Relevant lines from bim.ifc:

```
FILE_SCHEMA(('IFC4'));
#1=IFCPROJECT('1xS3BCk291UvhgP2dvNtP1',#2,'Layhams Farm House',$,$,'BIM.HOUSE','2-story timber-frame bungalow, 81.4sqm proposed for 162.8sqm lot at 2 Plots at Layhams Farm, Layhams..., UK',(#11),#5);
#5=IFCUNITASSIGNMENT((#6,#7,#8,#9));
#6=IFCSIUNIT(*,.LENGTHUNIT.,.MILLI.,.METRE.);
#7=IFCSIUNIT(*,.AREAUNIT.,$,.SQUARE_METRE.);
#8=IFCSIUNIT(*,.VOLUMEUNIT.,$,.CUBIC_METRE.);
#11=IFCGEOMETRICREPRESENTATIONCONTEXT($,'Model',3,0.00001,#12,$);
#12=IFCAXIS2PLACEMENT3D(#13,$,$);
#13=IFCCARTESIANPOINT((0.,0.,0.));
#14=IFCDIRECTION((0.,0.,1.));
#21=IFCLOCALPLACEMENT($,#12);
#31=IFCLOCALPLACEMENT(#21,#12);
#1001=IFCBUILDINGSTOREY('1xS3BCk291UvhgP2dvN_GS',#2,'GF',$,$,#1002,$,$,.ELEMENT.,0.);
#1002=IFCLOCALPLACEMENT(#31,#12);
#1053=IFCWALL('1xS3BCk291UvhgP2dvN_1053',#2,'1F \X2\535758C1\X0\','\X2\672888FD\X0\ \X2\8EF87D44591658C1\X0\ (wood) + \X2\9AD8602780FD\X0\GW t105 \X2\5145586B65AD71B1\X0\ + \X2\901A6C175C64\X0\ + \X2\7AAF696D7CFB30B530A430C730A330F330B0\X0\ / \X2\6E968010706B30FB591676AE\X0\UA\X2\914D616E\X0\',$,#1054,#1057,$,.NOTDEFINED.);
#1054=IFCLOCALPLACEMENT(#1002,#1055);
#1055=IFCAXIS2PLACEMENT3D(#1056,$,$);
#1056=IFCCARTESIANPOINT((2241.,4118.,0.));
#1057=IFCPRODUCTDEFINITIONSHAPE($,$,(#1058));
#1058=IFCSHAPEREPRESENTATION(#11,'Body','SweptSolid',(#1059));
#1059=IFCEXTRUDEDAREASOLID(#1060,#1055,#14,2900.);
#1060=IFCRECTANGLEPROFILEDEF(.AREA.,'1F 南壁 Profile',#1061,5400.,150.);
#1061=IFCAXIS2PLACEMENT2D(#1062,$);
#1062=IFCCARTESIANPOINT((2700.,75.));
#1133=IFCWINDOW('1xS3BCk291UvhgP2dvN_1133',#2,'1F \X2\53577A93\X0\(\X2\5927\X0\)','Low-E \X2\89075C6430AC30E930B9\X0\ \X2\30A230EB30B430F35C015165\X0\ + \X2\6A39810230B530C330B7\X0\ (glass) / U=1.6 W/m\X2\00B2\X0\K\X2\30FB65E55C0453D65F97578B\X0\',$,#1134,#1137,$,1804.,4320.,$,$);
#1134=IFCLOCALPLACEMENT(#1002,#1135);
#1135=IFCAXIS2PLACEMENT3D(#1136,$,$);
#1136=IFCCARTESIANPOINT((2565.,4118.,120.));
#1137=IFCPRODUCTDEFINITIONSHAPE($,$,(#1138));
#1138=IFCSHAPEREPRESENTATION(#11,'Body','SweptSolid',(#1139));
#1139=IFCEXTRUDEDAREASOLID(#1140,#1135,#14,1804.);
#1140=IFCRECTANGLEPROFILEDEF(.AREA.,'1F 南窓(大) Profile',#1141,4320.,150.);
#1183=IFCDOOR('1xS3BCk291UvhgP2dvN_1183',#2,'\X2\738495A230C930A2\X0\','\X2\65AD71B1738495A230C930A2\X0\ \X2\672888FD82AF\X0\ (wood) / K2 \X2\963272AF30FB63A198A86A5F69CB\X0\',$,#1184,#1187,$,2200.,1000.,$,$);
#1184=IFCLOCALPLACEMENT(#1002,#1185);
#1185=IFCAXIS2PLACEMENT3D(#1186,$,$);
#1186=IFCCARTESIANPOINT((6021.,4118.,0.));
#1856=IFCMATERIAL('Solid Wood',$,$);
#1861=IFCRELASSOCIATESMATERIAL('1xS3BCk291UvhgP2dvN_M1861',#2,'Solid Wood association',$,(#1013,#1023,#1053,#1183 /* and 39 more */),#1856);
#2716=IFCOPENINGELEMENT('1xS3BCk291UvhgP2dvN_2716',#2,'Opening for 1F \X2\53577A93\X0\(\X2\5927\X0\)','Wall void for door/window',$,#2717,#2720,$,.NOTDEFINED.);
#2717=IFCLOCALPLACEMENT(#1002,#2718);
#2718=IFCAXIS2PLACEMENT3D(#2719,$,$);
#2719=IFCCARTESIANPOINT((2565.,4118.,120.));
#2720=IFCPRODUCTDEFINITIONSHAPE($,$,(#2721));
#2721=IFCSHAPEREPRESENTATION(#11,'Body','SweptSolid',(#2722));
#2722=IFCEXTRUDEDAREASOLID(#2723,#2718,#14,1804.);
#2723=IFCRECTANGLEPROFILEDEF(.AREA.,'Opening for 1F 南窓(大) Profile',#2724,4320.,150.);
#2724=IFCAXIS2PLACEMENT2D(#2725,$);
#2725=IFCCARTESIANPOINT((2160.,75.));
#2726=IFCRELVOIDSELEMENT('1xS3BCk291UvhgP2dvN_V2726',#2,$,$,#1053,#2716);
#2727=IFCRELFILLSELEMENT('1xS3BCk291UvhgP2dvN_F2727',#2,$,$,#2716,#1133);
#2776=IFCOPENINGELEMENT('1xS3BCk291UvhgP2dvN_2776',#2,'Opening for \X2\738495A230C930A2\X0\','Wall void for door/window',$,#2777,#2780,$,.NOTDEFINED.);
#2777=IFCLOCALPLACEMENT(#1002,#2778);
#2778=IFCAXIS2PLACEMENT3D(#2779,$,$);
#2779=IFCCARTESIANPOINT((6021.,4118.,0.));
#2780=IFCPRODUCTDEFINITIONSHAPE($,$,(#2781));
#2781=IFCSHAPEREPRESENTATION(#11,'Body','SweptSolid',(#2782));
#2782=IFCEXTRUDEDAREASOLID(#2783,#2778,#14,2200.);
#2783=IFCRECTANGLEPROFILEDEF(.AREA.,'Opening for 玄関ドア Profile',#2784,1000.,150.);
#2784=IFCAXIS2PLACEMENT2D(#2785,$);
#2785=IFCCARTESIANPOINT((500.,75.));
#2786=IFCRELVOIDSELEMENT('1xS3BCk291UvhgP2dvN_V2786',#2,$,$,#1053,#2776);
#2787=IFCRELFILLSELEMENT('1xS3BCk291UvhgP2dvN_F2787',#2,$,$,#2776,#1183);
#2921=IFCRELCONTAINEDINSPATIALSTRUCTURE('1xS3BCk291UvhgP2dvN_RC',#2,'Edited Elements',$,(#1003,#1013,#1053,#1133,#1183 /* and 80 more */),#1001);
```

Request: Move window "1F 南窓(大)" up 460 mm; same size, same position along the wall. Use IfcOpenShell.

```python
import numpy as np
import ifcopenshell
import ifcopenshell.api.geometry
import ifcopenshell.util.placement
import ifcopenshell.util.unit

model = ifcopenshell.open("bim.ifc")
unit_scale = ifcopenshell.util.unit.calculate_unit_scale(model)

window = model.by_guid("1xS3BCk291UvhgP2dvN_1133")
opening = window.FillsVoids[0].RelatingOpeningElement
dz = 0.46 / unit_scale

shift = np.array([0.0, 0.0, dz])
# The window is not placed relative to its opening, so move both.
for product in (opening, window):
    matrix = ifcopenshell.util.placement.get_local_placement(product.ObjectPlacement)
    matrix[:3, 3] += shift
    ifcopenshell.api.geometry.edit_object_placement(model, product=product, matrix=matrix, is_si=False)

print(f"moved by {dz * unit_scale:+.3f} m")

model.write("bim-out.ifc")
```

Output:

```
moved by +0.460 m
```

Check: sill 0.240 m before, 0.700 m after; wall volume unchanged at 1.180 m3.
